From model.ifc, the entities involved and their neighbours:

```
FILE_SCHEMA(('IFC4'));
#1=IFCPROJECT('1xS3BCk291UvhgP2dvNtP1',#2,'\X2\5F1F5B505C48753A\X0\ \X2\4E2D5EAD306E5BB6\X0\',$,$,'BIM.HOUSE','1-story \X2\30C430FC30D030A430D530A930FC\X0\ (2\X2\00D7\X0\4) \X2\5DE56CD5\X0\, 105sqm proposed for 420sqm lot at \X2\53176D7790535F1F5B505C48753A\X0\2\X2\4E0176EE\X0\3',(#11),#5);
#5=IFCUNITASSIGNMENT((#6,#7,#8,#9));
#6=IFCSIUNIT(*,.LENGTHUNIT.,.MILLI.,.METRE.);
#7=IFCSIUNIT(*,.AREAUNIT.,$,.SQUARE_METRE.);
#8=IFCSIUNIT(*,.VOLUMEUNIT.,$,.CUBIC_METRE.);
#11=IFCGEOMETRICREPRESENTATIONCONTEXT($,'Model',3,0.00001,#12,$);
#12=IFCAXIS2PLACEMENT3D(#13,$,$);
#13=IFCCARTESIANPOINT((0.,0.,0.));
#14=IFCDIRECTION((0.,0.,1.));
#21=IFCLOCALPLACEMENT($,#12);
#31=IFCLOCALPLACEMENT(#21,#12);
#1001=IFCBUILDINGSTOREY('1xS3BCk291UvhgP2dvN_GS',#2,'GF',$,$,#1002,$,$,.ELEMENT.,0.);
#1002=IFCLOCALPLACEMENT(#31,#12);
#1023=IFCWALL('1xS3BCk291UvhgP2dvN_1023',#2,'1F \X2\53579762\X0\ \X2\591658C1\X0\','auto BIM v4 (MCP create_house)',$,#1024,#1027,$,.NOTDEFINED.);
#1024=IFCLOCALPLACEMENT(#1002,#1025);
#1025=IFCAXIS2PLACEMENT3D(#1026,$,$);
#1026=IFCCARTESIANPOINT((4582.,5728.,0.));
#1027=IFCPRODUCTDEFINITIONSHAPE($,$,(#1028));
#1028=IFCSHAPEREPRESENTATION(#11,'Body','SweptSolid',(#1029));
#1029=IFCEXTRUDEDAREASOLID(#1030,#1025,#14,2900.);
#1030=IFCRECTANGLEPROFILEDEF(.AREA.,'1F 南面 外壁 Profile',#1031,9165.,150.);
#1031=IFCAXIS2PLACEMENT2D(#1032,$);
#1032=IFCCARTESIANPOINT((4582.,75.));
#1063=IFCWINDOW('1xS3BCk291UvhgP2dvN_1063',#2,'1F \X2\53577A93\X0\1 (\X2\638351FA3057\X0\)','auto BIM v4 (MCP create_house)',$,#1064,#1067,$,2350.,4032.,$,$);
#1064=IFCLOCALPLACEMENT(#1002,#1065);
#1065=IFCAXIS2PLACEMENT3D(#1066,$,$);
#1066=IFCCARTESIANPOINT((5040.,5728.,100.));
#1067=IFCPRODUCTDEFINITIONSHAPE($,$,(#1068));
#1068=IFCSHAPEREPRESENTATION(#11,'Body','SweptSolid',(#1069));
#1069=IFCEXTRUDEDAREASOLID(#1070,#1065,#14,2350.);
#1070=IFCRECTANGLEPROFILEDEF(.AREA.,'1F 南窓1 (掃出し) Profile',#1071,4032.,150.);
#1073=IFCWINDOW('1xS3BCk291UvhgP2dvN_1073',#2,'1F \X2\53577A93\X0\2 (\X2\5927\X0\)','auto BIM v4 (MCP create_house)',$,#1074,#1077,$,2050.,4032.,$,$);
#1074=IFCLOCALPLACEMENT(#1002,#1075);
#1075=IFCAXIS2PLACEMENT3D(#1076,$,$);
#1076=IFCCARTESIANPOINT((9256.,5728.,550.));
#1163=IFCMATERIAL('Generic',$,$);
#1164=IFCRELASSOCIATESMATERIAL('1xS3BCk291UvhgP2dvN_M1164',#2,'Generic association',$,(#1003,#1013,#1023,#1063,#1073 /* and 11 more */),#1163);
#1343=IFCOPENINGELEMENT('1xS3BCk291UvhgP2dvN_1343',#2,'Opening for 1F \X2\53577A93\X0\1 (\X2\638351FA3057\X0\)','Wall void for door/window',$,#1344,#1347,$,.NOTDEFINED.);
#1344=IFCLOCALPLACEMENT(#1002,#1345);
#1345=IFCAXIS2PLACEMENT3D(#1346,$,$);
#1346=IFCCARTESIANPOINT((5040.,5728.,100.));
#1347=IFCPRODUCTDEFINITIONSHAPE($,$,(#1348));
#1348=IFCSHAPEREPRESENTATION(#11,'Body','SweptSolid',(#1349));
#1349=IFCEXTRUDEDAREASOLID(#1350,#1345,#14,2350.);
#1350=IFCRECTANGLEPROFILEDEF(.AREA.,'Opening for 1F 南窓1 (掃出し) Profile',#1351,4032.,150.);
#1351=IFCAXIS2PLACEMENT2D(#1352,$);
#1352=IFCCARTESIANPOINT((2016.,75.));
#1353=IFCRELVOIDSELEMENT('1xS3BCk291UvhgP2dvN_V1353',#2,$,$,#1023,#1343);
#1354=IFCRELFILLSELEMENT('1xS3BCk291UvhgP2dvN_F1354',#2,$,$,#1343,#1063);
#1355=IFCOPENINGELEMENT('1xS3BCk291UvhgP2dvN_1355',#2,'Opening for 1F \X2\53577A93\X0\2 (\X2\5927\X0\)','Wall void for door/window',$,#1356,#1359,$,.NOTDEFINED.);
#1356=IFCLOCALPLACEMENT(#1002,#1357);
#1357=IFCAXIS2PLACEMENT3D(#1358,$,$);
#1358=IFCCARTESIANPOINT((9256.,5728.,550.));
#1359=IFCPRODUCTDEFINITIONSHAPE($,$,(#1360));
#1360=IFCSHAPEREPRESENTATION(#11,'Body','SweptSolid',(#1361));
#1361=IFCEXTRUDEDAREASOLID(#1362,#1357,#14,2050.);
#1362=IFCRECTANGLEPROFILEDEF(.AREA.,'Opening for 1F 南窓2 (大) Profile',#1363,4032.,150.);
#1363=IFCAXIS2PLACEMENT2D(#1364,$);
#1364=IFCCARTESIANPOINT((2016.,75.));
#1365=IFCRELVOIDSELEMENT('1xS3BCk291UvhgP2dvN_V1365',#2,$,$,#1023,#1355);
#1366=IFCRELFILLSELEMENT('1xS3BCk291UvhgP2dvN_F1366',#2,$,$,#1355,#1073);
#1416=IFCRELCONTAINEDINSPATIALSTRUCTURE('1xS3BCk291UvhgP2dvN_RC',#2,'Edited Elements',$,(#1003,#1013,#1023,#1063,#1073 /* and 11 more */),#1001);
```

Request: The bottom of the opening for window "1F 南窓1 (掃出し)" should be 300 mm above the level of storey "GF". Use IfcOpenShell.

```python
import numpy as np
import ifcopenshell
import ifcopenshell.api.geometry
import ifcopenshell.geom
import ifcopenshell.util.element
import ifcopenshell.util.placement
import ifcopenshell.util.shape
import ifcopenshell.util.unit

model = ifcopenshell.open("model.ifc")
unit_scale = ifcopenshell.util.unit.calculate_unit_scale(model)

window = model.by_id(1063)
opening = window.FillsVoids[0].RelatingOpeningElement
storey = ifcopenshell.util.element.get_container(window, ifc_class="IfcBuildingStorey")
level = ifcopenshell.util.placement.get_local_placement(storey.ObjectPlacement)[2, 3]

# The opening's origin need not be at the sill, so measure its lowest point.
shape = ifcopenshell.geom.create_shape(ifcopenshell.geom.settings(), opening)
bottom = ifcopenshell.util.shape.get_shape_bottom_elevation(shape, shape.geometry) / unit_scale
dz = level + 300.0 - bottom

shift = np.array([0.0, 0.0, dz])
# The window is not placed relative to its opening, so move both.
for product in (opening, window):
    matrix = ifcopenshell.util.placement.get_local_placement(product.ObjectPlacement)
    matrix[:3, 3] += shift
    ifcopenshell.api.geometry.edit_object_placement(model, product=product, matrix=matrix, is_si=False)

print(f"moved by {dz * unit_scale:+.3f} m")

model.write("model-out.ifc")
```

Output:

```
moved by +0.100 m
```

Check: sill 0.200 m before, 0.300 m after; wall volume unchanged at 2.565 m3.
